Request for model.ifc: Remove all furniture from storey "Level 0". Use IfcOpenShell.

First a look at what the model holds.

```python
import ifcopenshell
import ifcopenshell.util.element

model = ifcopenshell.open("model.ifc")
print(model.schema)
storey = next(s for s in model.by_type("IfcBuildingStorey") if s.Name == "Level 0")
furniture = [e for e in ifcopenshell.util.element.get_decomposition(storey) if e.is_a("IfcFurnishingElement")]
seen = {}
for e in furniture:
    element_type = ifcopenshell.util.element.get_type(e)
    name = element_type.Name if element_type not in (None, e) else None
    seen[name] = seen.get(name, 0) + 1
for name, count in sorted(seen.items(), key=str):
    print(count, "x", name)
```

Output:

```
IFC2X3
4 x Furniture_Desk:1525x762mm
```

```python
import ifcopenshell
import ifcopenshell.api.root
import ifcopenshell.util.element

model = ifcopenshell.open("model.ifc")

storey = next(s for s in model.by_type("IfcBuildingStorey") if s.Name == "Level 0")
furniture = [e for e in ifcopenshell.util.element.get_decomposition(storey) if e.is_a("IfcFurnishingElement")]

for e in furniture:
    ifcopenshell.api.root.remove_product(model, product=e)
print(len(furniture), "removed")

model.write("model-out.ifc")
```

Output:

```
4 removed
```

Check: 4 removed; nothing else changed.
